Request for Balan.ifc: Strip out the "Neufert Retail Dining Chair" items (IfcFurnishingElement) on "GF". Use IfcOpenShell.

First a look at what the model holds.

```python
import ifcopenshell
import ifcopenshell.util.element

model = ifcopenshell.open("Balan.ifc")
print(model.schema)
storey = next(s for s in model.by_type("IfcBuildingStorey") if s.Name == "GF")
furniture = [e for e in ifcopenshell.util.element.get_decomposition(storey) if e.is_a("IfcFurnishingElement")]
seen = {}
for e in furniture:
    element_type = ifcopenshell.util.element.get_type(e)
    name = element_type.Name if element_type not in (None, e) else None
    seen[name] = seen.get(name, 0) + 1
for name, count in sorted(seen.items(), key=str):
    print(count, "x", name)
```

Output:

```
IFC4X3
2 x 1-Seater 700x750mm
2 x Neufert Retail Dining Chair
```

```python
import ifcopenshell
import ifcopenshell.api.root
import ifcopenshell.util.element

model = ifcopenshell.open("Balan.ifc")

storey = next(s for s in model.by_type("IfcBuildingStorey") if s.Name == "GF")
furniture = [e for e in ifcopenshell.util.element.get_decomposition(storey) if e.is_a("IfcFurnishingElement")]
targets = [e for e in furniture if (t := ifcopenshell.util.element.get_type(e)) not in (None, e) and t.Name == "Neufert Retail Dining Chair"]

for e in targets:
    ifcopenshell.api.root.remove_product(model, product=e)
print(len(targets), "removed")

model.write("Balan_edited.ifc")
```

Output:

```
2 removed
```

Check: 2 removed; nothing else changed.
